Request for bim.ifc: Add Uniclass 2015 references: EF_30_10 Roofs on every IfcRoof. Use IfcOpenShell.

First a look at what the model holds.

```python
import ifcopenshell

model = ifcopenshell.open("bim.ifc")
print(model.schema)
print("classifications:", [c.Name for c in model.by_type("IfcClassification")])
for ifc_class in ("IfcDoor", "IfcRoof", "IfcStair", "IfcWall", "IfcWindow"):
    print(ifc_class, len(model.by_type(ifc_class)))
```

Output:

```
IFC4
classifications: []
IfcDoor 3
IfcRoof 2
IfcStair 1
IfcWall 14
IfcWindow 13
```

```python
import ifcopenshell
import ifcopenshell.api.classification

model = ifcopenshell.open("bim.ifc")

system = ifcopenshell.api.classification.add_classification(model, classification="Uniclass 2015")

codes = {
    "IfcRoof": ("EF_30_10", "Roofs"),
}
for ifc_class, (code, name) in codes.items():
    products = model.by_type(ifc_class)
    ifcopenshell.api.classification.add_reference(
        model, products=products, classification=system, identification=code, name=name
    )
    print(code, len(products))

model.write("bim-out.ifc")
```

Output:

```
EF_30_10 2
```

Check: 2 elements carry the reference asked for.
